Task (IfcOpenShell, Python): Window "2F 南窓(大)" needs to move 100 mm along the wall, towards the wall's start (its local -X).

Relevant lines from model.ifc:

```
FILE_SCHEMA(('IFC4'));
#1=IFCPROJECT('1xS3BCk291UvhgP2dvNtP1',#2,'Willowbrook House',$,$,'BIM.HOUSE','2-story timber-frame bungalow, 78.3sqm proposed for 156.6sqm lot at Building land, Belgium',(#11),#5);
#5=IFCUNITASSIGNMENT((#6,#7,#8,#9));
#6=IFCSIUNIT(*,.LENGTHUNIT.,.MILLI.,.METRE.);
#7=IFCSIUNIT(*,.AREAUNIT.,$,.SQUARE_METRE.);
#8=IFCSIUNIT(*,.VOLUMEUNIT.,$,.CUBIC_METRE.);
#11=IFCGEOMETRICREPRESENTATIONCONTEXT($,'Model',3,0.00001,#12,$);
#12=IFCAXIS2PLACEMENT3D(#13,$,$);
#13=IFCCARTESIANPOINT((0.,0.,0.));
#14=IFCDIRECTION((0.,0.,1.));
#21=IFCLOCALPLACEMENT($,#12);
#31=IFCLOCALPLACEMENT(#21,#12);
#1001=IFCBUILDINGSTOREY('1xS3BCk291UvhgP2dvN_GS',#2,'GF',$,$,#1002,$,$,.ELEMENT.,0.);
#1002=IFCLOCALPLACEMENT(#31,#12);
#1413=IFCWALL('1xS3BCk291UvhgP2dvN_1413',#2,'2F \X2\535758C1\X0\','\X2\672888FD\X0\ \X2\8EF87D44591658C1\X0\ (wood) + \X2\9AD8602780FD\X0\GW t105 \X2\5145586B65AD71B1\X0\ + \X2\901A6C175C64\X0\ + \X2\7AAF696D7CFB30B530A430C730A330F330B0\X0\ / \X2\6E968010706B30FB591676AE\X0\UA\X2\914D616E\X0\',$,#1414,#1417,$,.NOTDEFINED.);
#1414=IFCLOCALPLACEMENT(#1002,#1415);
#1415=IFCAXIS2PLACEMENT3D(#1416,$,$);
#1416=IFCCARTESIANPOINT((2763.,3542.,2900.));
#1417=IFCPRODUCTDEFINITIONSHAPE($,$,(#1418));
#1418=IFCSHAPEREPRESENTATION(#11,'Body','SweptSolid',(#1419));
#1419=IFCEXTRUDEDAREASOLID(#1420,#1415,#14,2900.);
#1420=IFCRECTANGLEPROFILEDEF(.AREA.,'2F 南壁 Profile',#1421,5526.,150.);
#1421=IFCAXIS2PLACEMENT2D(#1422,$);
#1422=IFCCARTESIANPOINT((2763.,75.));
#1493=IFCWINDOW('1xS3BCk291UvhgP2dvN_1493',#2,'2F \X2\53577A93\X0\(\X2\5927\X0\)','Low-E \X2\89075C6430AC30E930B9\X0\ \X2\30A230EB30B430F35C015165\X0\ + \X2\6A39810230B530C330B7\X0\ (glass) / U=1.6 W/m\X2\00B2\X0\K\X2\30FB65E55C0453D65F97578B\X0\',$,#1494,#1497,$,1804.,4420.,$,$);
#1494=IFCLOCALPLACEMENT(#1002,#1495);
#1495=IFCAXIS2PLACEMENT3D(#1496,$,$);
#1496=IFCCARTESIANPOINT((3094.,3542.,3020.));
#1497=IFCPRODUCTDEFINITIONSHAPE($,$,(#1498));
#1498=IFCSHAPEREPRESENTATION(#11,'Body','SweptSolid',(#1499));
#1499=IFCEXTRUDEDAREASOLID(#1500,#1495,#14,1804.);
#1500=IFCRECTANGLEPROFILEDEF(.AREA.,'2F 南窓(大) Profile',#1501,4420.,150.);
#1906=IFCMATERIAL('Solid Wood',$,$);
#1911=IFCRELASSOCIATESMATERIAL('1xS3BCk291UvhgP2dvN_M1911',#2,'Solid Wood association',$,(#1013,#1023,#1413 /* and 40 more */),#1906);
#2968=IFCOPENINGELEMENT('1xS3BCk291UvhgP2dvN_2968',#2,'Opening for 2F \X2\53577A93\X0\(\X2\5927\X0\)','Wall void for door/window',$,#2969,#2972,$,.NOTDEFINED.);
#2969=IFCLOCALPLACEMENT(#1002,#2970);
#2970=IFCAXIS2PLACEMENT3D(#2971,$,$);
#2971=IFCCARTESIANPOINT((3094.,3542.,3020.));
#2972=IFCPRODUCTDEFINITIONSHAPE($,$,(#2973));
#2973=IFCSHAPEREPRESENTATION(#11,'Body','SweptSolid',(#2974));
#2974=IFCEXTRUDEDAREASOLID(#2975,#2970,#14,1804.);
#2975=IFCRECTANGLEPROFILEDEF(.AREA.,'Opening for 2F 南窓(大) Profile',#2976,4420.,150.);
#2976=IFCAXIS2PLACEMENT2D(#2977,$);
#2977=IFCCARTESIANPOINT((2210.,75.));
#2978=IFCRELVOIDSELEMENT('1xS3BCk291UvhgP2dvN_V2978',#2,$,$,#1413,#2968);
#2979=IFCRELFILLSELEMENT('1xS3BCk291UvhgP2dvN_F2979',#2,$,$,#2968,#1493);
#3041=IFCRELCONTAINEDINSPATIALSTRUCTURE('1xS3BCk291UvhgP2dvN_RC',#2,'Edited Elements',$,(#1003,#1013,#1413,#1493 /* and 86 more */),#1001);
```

```python
import ifcopenshell
import ifcopenshell.api.geometry
import ifcopenshell.util.placement

model = ifcopenshell.open("model.ifc")

window = model.by_guid("1xS3BCk291UvhgP2dvN_1493")
opening = window.FillsVoids[0].RelatingOpeningElement
wall = opening.VoidsElements[0].RelatingBuildingElement

wall_matrix = ifcopenshell.util.placement.get_local_placement(wall.ObjectPlacement)
shift = wall_matrix[:3, 0] * -100.0
before = ifcopenshell.util.placement.get_local_placement(window.ObjectPlacement)[:3, 3].copy()

# The window is not placed relative to its opening, so move both.
for product in (opening, window):
    matrix = ifcopenshell.util.placement.get_local_placement(product.ObjectPlacement)
    matrix[:3, 3] += shift
    ifcopenshell.api.geometry.edit_object_placement(model, product=product, matrix=matrix, is_si=False)

after = ifcopenshell.util.placement.get_local_placement(window.ObjectPlacement)[:3, 3]
print("window moved by", (after - before).round(3) + 0.0)

model.write("model_rev.ifc")
```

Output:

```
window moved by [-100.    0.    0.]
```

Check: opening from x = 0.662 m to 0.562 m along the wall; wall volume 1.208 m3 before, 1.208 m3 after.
